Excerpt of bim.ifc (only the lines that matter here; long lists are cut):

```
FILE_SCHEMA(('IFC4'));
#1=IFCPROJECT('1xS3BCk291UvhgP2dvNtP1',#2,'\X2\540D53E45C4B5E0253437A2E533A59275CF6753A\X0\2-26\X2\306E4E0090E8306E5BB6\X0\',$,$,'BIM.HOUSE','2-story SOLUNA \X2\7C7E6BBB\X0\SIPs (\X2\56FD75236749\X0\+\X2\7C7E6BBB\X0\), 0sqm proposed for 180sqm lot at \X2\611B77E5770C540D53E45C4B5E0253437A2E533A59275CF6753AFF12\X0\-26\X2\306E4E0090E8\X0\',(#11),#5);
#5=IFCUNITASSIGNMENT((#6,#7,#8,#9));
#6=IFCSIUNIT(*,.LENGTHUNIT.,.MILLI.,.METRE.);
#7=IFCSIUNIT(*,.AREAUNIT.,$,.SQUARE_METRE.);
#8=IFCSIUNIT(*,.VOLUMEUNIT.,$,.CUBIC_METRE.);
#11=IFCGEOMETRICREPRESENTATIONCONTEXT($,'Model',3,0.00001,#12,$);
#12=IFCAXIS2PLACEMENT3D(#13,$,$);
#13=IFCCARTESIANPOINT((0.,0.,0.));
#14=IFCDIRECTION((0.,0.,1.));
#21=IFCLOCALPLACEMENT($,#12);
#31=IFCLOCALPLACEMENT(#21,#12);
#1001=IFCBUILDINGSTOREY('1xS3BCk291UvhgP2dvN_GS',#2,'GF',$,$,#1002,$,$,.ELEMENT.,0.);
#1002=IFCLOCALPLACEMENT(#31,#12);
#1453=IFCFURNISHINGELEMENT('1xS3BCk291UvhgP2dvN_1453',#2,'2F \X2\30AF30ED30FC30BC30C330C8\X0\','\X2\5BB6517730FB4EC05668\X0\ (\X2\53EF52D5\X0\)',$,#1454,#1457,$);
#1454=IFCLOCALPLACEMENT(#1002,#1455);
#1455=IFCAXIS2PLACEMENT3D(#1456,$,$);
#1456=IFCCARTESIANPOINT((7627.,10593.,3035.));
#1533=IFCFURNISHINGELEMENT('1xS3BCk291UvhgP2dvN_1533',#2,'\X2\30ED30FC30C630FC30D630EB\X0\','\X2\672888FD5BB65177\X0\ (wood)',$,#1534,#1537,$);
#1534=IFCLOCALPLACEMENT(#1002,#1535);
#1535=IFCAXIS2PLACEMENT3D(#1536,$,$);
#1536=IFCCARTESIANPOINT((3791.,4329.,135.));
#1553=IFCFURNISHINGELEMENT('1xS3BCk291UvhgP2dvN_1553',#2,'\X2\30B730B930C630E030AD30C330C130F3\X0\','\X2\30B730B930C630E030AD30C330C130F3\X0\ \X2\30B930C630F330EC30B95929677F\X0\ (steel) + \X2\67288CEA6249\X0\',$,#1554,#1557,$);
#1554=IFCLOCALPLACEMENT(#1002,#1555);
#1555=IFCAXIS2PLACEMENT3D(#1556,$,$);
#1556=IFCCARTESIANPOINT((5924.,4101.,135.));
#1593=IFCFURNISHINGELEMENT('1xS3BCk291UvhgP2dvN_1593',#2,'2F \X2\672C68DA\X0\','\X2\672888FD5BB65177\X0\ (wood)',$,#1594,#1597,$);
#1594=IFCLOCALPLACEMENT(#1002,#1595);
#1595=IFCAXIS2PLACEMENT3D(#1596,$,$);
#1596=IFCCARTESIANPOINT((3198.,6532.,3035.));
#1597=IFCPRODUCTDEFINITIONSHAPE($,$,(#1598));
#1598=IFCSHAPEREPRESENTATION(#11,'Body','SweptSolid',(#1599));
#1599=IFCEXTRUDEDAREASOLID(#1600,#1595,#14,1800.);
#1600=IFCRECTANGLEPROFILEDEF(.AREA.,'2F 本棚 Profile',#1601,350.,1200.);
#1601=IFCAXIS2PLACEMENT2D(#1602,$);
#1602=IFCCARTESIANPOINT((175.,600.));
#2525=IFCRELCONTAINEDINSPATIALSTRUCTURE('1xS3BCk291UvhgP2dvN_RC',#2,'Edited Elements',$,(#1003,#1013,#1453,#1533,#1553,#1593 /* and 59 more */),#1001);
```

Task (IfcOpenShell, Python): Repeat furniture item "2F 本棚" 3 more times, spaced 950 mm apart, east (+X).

```python
import numpy as np
import ifcopenshell
import ifcopenshell.api.geometry
import ifcopenshell.api.root
import ifcopenshell.util.element
import ifcopenshell.util.placement

model = ifcopenshell.open("bim.ifc")


def reuse_history(source, copy):
    """copy_class also copies each property set's owner history, people and application; keep the originals."""
    for rel in copy.IsDefinedBy:
        if rel.is_a("IfcRelDefinesByProperties") and (history := rel.RelatingPropertyDefinition.OwnerHistory):
            rel.RelatingPropertyDefinition.OwnerHistory = source.OwnerHistory
            ifcopenshell.util.element.remove_deep2(model, history)


source = model.by_id(1593)
base = ifcopenshell.util.placement.get_local_placement(source.ObjectPlacement)
step = np.array([1.0, 0.0, 0.0]) * 950.0

for i in range(1, 4):
    copy = ifcopenshell.api.root.copy_class(model, product=source)
    copy.Representation = ifcopenshell.util.element.copy_deep(
        model, source.Representation, exclude=["IfcGeometricRepresentationContext", "IfcRepresentationMap"]
    )
    reuse_history(source, copy)
    matrix = base.copy()
    matrix[:3, 3] += i * step
    print("added at", matrix[:3, 3].round(3) + 0.0)
    ifcopenshell.api.geometry.edit_object_placement(model, product=copy, matrix=matrix, is_si=False)

model.write("bim_rev.ifc")
```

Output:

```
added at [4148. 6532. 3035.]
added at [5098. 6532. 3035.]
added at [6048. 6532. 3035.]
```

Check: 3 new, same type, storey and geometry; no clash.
